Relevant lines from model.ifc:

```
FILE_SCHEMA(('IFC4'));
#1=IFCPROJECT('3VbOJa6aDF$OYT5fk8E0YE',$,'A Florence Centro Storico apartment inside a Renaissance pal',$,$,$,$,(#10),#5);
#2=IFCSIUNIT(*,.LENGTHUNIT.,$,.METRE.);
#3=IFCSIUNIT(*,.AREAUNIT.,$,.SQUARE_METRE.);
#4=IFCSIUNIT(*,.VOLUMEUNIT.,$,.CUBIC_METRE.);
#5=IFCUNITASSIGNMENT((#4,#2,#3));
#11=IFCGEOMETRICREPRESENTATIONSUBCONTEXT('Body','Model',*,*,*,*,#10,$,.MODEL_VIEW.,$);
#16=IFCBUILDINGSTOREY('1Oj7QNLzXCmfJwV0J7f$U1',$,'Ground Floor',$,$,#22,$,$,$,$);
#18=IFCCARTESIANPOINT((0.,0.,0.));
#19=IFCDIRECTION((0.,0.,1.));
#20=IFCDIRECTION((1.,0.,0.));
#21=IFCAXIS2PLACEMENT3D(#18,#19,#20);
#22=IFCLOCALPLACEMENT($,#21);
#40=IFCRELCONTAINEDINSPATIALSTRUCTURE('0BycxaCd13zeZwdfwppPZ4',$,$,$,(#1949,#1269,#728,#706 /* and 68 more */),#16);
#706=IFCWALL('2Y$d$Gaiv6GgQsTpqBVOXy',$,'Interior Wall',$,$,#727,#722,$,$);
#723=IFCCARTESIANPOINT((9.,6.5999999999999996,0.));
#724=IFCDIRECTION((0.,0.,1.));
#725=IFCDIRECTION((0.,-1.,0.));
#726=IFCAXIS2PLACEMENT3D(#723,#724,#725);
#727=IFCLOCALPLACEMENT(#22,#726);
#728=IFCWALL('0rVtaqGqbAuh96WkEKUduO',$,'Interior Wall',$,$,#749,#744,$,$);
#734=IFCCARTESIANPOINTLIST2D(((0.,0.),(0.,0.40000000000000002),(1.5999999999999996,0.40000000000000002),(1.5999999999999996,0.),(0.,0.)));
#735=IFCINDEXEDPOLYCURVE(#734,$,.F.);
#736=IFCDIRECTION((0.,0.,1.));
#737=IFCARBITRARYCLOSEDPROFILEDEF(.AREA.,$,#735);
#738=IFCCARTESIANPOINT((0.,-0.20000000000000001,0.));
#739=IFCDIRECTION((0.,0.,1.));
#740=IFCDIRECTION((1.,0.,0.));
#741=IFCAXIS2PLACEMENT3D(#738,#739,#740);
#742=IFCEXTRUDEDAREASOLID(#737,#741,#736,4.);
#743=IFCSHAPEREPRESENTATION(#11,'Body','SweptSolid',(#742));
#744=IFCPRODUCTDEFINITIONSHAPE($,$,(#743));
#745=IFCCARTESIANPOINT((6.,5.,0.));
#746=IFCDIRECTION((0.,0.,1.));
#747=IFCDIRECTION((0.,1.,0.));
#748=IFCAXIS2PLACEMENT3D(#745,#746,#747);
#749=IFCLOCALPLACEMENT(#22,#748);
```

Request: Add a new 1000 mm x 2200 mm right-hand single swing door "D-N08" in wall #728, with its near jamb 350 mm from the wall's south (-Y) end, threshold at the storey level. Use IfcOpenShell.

```python
import numpy as np
import ifcopenshell
import ifcopenshell.api.feature
import ifcopenshell.api.geometry
import ifcopenshell.api.root
import ifcopenshell.api.spatial
import ifcopenshell.geom
import ifcopenshell.util.element
import ifcopenshell.util.placement
import ifcopenshell.util.representation
import ifcopenshell.util.shape
import ifcopenshell.util.unit

model = ifcopenshell.open("model.ifc")
unit_scale = ifcopenshell.util.unit.calculate_unit_scale(model)
settings = ifcopenshell.geom.settings()


def volume(element):
    """Net volume in cubic metres, openings subtracted."""
    shape = ifcopenshell.geom.create_shape(settings, element)
    return ifcopenshell.util.shape.get_volume(shape.geometry)


wall = model.by_guid("0rVtaqGqbAuh96WkEKUduO")
storey = ifcopenshell.util.element.get_container(wall, ifc_class="IfcBuildingStorey")
context = ifcopenshell.util.representation.get_context(model, "Model", "Body", "MODEL_VIEW")
before = volume(wall)

width, height, from_end, sill = 1, 2.2, 0.35, 0.0  # metres

# The wall runs along its own X axis, and the end named is its -X end.
wall_shape = ifcopenshell.geom.create_shape(settings, wall)
x, y, z = ifcopenshell.util.shape.get_vertices(wall_shape.geometry).T
start = x.min() + from_end
face, thickness = float(y.min()), float(y.max() - y.min())
wall_matrix = ifcopenshell.util.placement.get_local_placement(wall.ObjectPlacement)
level = ifcopenshell.util.placement.get_local_placement(storey.ObjectPlacement)[2, 3]


def in_wall(x, y):
    """Placement at x, y metres in the wall's axes, at sill height."""
    matrix = wall_matrix.copy()
    matrix[:, 3] = wall_matrix @ np.array([x / unit_scale, y / unit_scale, 0.0, 1.0])
    matrix[2, 3] = level + sill / unit_scale
    return matrix


# Opening: a box that overshoots both wall faces by 50 mm.
opening = ifcopenshell.api.root.create_entity(model, ifc_class="IfcOpeningElement", predefined_type="OPENING")
box = ifcopenshell.api.geometry.add_wall_representation(
    model, context=context, length=width, height=height, thickness=thickness + 0.1
)
ifcopenshell.api.geometry.assign_representation(model, product=opening, representation=box)
ifcopenshell.api.geometry.edit_object_placement(model, product=opening, matrix=in_wall(start, face - 0.05), is_si=False)
ifcopenshell.api.feature.add_feature(model, feature=opening, element=wall)

door = ifcopenshell.api.root.create_entity(model, ifc_class="IfcDoor", name="D-N08", predefined_type="DOOR")
door.OverallWidth, door.OverallHeight = width / unit_scale, height / unit_scale
door.OperationType = "SINGLE_SWING_RIGHT"
body = ifcopenshell.api.geometry.add_door_representation(
    model,
    context=context,
    overall_width=door.OverallWidth,
    overall_height=door.OverallHeight,
    operation_type="SINGLE_SWING_RIGHT",
    lining_properties={"LiningDepth": thickness / unit_scale, "ThresholdDepth": thickness / unit_scale},
)
ifcopenshell.api.geometry.assign_representation(model, product=door, representation=body)
ifcopenshell.api.spatial.assign_container(model, products=[door], relating_structure=storey)
ifcopenshell.api.feature.add_filling(model, opening=opening, element=door)

# The lining spans the wall, so the door starts at the wall face.
ifcopenshell.api.geometry.edit_object_placement(model, product=door, matrix=in_wall(start, face), is_si=False)

after = volume(wall)

print(f"wall volume {before:.3f} -> {after:.3f} m3")

model.write("model_updated.ifc")
```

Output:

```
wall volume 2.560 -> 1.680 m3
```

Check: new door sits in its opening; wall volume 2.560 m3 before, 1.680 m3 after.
